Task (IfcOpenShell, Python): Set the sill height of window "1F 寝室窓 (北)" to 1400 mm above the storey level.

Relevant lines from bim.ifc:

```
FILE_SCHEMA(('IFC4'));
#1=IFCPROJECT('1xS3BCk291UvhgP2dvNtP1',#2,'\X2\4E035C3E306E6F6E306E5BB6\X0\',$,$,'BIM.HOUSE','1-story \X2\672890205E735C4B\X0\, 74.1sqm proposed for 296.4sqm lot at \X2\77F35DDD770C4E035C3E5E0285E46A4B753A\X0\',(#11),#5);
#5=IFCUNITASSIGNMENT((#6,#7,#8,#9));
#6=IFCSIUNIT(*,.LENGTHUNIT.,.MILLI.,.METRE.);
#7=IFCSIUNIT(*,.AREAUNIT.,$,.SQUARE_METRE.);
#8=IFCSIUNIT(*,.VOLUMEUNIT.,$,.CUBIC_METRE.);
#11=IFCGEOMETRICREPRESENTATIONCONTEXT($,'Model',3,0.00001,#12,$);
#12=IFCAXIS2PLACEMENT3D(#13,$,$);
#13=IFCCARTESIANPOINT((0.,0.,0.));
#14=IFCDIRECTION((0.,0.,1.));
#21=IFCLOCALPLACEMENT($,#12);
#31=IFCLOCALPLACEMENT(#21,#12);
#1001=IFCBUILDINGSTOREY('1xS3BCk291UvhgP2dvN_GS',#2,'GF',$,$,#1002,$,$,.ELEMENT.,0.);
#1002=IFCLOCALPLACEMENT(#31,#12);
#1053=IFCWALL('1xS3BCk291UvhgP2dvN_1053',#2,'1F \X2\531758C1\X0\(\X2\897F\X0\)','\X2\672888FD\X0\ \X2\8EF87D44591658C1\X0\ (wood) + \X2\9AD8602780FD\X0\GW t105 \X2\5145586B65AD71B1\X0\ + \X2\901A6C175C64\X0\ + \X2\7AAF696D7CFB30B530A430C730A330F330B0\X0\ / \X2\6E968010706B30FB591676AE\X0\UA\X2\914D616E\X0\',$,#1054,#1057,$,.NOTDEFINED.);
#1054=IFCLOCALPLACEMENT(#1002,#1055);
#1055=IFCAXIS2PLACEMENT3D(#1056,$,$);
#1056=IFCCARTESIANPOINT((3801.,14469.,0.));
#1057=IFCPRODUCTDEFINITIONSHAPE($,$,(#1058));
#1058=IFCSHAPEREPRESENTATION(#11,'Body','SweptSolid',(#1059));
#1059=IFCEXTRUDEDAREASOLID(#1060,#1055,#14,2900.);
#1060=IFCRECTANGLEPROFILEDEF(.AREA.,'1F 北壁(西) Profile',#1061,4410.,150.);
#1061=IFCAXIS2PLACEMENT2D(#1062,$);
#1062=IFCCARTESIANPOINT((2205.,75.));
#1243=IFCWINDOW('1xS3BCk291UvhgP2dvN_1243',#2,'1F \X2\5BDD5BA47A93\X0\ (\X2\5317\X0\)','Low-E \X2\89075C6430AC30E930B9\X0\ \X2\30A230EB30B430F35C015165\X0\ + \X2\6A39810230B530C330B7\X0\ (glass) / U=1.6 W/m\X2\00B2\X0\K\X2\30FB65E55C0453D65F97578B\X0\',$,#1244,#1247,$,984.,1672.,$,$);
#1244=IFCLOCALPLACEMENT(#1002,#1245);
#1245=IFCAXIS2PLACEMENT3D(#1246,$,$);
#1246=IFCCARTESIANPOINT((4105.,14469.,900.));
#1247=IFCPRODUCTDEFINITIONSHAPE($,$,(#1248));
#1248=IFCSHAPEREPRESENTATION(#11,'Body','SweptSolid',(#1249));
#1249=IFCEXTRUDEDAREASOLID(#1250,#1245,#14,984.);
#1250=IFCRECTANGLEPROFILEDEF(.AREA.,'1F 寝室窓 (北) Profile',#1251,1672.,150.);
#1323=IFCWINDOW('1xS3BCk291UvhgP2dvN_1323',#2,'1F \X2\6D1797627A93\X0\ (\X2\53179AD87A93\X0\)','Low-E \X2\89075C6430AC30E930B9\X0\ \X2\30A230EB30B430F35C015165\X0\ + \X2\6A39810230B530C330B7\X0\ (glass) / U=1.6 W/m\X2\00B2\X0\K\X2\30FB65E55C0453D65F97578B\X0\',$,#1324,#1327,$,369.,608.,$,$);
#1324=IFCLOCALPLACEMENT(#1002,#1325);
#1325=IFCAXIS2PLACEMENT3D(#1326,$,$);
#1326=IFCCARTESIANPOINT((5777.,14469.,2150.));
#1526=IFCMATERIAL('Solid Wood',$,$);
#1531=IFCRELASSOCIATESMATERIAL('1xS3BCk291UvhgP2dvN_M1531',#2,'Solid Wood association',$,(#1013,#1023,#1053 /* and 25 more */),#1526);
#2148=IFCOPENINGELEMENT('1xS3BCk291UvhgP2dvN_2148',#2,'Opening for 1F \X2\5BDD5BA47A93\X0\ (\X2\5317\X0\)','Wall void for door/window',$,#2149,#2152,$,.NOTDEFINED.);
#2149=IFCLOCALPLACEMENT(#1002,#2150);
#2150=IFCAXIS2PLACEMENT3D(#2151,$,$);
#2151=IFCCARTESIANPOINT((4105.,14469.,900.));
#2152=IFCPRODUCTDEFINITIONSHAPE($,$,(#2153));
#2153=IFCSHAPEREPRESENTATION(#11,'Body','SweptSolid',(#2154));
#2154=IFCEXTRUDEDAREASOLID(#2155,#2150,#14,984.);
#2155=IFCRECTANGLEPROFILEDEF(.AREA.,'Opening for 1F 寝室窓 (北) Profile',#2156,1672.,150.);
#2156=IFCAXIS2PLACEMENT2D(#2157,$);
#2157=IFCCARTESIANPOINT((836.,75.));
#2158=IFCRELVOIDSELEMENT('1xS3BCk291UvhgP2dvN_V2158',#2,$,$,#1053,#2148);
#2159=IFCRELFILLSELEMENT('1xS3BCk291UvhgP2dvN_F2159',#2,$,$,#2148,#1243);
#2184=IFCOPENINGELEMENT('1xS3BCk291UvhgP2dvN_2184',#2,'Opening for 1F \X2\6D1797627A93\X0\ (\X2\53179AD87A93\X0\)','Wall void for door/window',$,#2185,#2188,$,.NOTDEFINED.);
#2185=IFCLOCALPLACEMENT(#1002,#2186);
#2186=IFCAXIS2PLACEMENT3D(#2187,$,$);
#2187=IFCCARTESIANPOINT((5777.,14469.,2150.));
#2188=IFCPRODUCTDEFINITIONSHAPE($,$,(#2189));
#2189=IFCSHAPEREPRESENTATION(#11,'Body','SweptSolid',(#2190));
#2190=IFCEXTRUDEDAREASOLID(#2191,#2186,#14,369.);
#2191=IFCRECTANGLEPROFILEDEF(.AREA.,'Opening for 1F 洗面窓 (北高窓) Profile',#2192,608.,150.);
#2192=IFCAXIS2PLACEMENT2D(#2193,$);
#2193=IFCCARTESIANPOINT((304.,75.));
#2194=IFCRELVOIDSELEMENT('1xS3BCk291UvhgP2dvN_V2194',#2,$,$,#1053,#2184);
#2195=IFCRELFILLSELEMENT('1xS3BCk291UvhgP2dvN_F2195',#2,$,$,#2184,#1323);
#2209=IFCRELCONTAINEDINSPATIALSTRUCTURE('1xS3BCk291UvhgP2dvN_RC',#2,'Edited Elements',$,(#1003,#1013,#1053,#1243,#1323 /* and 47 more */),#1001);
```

```python
import numpy as np
import ifcopenshell
import ifcopenshell.api.geometry
import ifcopenshell.geom
import ifcopenshell.util.element
import ifcopenshell.util.placement
import ifcopenshell.util.shape
import ifcopenshell.util.unit

model = ifcopenshell.open("bim.ifc")
unit_scale = ifcopenshell.util.unit.calculate_unit_scale(model)

window = model.by_id(1243)
opening = window.FillsVoids[0].RelatingOpeningElement
storey = ifcopenshell.util.element.get_container(window, ifc_class="IfcBuildingStorey")
level = ifcopenshell.util.placement.get_local_placement(storey.ObjectPlacement)[2, 3]

# The opening's origin need not be at the sill, so measure its lowest point.
shape = ifcopenshell.geom.create_shape(ifcopenshell.geom.settings(), opening)
bottom = ifcopenshell.util.shape.get_shape_bottom_elevation(shape, shape.geometry) / unit_scale
dz = level + 1.4 / unit_scale - bottom

shift = np.array([0.0, 0.0, dz])
# The window is not placed relative to its opening, so move both.
for product in (opening, window):
    matrix = ifcopenshell.util.placement.get_local_placement(product.ObjectPlacement)
    matrix[:3, 3] += shift
    ifcopenshell.api.geometry.edit_object_placement(model, product=product, matrix=matrix, is_si=False)

print(f"moved by {dz * unit_scale:+.3f} m")

model.write("bim-out.ifc")
```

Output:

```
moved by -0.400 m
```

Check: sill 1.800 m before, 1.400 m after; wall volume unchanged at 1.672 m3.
